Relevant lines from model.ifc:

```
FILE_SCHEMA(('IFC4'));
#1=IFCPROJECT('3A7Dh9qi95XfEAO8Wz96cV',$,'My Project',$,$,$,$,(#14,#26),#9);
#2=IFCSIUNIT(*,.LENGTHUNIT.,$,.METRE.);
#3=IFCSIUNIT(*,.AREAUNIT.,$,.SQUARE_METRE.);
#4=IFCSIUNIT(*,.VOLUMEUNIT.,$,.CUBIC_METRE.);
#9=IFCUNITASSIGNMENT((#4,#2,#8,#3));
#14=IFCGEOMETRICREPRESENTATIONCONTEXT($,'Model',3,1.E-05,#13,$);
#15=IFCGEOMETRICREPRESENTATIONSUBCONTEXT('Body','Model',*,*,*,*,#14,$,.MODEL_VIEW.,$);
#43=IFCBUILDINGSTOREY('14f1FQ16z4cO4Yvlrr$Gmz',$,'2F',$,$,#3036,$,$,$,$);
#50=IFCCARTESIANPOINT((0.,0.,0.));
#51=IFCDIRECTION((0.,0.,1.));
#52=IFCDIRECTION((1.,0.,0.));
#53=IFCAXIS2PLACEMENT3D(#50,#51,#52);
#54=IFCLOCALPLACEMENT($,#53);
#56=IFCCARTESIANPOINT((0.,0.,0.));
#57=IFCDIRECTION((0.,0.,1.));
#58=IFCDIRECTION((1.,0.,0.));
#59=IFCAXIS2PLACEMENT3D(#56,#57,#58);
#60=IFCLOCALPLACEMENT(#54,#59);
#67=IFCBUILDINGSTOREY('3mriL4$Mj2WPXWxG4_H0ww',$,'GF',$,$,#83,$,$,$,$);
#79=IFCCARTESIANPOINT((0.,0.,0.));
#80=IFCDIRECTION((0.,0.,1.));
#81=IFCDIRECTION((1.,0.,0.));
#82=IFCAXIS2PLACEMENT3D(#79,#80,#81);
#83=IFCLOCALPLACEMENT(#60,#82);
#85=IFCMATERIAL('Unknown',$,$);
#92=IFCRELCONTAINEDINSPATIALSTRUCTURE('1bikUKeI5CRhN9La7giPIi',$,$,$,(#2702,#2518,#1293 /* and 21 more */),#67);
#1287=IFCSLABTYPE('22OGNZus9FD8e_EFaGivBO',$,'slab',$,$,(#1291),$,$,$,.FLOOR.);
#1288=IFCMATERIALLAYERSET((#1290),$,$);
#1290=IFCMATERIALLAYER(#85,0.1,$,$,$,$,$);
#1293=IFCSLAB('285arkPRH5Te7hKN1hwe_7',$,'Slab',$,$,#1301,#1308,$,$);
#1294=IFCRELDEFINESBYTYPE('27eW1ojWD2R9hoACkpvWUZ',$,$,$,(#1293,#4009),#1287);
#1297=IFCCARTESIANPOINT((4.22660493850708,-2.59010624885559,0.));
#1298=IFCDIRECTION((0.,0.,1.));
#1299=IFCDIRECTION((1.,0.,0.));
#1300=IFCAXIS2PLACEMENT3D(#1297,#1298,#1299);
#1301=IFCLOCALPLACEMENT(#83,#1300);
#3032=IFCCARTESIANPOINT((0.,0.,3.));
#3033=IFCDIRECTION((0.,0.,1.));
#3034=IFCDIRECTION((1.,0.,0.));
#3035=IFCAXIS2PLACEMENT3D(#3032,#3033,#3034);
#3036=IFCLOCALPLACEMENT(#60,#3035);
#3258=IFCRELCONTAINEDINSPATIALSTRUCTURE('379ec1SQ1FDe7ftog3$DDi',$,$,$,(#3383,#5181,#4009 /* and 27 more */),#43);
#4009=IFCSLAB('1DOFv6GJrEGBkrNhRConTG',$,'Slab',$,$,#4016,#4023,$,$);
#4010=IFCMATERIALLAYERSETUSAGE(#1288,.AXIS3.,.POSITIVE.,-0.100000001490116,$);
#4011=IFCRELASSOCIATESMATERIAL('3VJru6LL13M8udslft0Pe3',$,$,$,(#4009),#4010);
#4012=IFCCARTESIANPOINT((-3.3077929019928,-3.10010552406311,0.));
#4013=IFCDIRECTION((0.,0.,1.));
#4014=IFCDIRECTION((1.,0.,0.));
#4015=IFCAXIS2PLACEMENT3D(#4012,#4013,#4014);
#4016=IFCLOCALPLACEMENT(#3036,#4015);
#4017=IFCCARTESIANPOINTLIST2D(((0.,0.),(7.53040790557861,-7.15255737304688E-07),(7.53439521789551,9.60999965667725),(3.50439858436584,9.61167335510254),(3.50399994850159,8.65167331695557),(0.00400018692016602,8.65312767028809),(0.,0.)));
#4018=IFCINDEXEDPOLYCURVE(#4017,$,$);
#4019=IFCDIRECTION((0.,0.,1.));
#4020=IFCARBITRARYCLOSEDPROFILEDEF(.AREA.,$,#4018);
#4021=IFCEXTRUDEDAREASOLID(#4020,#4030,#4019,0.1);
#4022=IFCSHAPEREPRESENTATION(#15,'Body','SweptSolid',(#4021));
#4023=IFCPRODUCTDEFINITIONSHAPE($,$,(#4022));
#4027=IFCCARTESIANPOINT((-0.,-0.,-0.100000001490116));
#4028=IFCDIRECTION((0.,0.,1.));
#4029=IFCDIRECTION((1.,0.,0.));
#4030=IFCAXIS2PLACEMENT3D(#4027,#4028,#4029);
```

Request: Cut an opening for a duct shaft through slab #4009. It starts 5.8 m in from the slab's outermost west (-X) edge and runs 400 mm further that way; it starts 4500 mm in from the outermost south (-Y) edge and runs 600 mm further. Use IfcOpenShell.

```python
import numpy as np
import ifcopenshell
import ifcopenshell.api.feature
import ifcopenshell.api.geometry
import ifcopenshell.api.root
import ifcopenshell.geom
import ifcopenshell.util.placement
import ifcopenshell.util.representation
import ifcopenshell.util.shape
import ifcopenshell.util.unit

model = ifcopenshell.open("model.ifc")
unit_scale = ifcopenshell.util.unit.calculate_unit_scale(model)
settings = ifcopenshell.geom.settings()


def volume(element):
    """Net volume in cubic metres, openings subtracted."""
    shape = ifcopenshell.geom.create_shape(settings, element)
    return ifcopenshell.util.shape.get_volume(shape.geometry)


slab = model.by_id(4009)
before = volume(slab)

# Extent in the slab's own axes, in metres. The edges named are its -X and -Y sides.
slab_shape = ifcopenshell.geom.create_shape(settings, slab)
vertices = ifcopenshell.util.shape.get_vertices(slab_shape.geometry)
x_min, y_min, bottom = vertices.min(axis=0)
top = vertices[:, 2].max()

opening = ifcopenshell.api.root.create_entity(model, ifc_class="IfcOpeningElement", name="Duct shaft opening", predefined_type="OPENING")
context = ifcopenshell.util.representation.get_context(model, "Model", "Body", "MODEL_VIEW")
width, depth = 0.4, 0.6
outline = [(0.0, 0.0), (width, 0.0), (width, depth), (0.0, depth), (0.0, 0.0)]
# Overshoot both faces by 50 mm so the cut is clean.
shape = ifcopenshell.api.geometry.add_slab_representation(
    model, context=context, depth=top - bottom + 0.1, polyline=outline
)
ifcopenshell.api.geometry.assign_representation(model, product=opening, representation=shape)

matrix = ifcopenshell.util.placement.get_local_placement(slab.ObjectPlacement)
matrix[:, 3] = matrix @ np.append(np.array([x_min + 5.8, y_min + 4.5, bottom - 0.05]) / unit_scale, 1.0)
ifcopenshell.api.geometry.edit_object_placement(model, product=opening, matrix=matrix, is_si=False)
ifcopenshell.api.feature.add_feature(model, feature=opening, element=slab)

after = volume(slab)

print(f"slab volume {before:.3f} -> {after:.3f} m3")

model.write("model_updated.ifc")
```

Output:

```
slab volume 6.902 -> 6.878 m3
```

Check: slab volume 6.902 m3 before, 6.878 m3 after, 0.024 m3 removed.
